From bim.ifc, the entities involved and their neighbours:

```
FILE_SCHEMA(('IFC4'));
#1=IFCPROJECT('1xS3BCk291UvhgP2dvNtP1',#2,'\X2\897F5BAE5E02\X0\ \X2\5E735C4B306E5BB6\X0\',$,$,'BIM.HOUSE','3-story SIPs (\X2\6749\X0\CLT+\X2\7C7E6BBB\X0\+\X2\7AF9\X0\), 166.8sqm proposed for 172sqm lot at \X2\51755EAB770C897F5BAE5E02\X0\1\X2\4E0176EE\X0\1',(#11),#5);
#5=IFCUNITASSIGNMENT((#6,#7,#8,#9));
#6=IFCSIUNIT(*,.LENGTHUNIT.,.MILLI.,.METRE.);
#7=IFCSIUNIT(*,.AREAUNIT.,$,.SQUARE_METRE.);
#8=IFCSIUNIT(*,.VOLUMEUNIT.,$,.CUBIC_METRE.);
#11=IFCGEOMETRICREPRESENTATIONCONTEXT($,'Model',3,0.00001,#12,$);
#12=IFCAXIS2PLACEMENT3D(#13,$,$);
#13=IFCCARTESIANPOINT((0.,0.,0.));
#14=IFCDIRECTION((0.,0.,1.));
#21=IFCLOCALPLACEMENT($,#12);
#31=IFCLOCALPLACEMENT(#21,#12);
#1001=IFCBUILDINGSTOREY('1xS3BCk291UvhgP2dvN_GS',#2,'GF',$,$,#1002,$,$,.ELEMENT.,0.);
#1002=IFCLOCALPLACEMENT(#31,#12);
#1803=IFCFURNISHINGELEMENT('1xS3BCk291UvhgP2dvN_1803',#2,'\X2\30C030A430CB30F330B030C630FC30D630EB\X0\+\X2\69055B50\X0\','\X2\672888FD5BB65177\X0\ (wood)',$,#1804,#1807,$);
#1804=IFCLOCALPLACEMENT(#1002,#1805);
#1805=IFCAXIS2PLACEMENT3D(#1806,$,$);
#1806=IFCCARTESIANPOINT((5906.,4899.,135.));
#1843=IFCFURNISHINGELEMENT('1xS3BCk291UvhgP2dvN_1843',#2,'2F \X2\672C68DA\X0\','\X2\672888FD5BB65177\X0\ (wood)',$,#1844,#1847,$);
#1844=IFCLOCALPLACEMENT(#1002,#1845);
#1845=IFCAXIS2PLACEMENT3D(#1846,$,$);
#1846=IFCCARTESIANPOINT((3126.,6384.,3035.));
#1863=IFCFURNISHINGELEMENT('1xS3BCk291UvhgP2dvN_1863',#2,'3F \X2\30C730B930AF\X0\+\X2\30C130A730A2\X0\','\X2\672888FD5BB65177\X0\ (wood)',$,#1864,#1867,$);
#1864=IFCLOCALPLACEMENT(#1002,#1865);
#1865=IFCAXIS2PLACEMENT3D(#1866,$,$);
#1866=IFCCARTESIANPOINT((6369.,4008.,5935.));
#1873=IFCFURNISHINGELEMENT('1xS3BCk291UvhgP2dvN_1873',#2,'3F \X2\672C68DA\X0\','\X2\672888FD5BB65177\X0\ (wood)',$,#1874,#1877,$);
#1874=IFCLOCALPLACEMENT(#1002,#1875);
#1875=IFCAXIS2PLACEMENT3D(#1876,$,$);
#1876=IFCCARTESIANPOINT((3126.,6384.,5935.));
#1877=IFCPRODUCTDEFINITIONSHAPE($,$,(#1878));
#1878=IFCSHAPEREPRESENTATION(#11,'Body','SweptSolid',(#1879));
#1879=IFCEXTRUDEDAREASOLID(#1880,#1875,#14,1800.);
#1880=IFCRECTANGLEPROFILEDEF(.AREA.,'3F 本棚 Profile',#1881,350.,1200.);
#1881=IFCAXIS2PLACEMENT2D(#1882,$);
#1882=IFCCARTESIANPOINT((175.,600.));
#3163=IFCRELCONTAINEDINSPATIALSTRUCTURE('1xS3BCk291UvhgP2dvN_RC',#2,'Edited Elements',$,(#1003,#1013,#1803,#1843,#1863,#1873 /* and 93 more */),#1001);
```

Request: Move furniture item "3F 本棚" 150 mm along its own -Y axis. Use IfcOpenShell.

```python
import ifcopenshell
import ifcopenshell.api.geometry
import ifcopenshell.util.placement
import ifcopenshell.util.unit

model = ifcopenshell.open("bim.ifc")
unit_scale = ifcopenshell.util.unit.calculate_unit_scale(model)

item = model.by_id(1873)
matrix = ifcopenshell.util.placement.get_local_placement(item.ObjectPlacement)
matrix[:3, 3] -= matrix[:3, 1] * 0.15 / unit_scale
ifcopenshell.api.geometry.edit_object_placement(model, product=item, matrix=matrix, is_si=False)

print(ifcopenshell.util.placement.get_local_placement(item.ObjectPlacement).round(3) + 0.0)

model.write("bim_updated.ifc")
```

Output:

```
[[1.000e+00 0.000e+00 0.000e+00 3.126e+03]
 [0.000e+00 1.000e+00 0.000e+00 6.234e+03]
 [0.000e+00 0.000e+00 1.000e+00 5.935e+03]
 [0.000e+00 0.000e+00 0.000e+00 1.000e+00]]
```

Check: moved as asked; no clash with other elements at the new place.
